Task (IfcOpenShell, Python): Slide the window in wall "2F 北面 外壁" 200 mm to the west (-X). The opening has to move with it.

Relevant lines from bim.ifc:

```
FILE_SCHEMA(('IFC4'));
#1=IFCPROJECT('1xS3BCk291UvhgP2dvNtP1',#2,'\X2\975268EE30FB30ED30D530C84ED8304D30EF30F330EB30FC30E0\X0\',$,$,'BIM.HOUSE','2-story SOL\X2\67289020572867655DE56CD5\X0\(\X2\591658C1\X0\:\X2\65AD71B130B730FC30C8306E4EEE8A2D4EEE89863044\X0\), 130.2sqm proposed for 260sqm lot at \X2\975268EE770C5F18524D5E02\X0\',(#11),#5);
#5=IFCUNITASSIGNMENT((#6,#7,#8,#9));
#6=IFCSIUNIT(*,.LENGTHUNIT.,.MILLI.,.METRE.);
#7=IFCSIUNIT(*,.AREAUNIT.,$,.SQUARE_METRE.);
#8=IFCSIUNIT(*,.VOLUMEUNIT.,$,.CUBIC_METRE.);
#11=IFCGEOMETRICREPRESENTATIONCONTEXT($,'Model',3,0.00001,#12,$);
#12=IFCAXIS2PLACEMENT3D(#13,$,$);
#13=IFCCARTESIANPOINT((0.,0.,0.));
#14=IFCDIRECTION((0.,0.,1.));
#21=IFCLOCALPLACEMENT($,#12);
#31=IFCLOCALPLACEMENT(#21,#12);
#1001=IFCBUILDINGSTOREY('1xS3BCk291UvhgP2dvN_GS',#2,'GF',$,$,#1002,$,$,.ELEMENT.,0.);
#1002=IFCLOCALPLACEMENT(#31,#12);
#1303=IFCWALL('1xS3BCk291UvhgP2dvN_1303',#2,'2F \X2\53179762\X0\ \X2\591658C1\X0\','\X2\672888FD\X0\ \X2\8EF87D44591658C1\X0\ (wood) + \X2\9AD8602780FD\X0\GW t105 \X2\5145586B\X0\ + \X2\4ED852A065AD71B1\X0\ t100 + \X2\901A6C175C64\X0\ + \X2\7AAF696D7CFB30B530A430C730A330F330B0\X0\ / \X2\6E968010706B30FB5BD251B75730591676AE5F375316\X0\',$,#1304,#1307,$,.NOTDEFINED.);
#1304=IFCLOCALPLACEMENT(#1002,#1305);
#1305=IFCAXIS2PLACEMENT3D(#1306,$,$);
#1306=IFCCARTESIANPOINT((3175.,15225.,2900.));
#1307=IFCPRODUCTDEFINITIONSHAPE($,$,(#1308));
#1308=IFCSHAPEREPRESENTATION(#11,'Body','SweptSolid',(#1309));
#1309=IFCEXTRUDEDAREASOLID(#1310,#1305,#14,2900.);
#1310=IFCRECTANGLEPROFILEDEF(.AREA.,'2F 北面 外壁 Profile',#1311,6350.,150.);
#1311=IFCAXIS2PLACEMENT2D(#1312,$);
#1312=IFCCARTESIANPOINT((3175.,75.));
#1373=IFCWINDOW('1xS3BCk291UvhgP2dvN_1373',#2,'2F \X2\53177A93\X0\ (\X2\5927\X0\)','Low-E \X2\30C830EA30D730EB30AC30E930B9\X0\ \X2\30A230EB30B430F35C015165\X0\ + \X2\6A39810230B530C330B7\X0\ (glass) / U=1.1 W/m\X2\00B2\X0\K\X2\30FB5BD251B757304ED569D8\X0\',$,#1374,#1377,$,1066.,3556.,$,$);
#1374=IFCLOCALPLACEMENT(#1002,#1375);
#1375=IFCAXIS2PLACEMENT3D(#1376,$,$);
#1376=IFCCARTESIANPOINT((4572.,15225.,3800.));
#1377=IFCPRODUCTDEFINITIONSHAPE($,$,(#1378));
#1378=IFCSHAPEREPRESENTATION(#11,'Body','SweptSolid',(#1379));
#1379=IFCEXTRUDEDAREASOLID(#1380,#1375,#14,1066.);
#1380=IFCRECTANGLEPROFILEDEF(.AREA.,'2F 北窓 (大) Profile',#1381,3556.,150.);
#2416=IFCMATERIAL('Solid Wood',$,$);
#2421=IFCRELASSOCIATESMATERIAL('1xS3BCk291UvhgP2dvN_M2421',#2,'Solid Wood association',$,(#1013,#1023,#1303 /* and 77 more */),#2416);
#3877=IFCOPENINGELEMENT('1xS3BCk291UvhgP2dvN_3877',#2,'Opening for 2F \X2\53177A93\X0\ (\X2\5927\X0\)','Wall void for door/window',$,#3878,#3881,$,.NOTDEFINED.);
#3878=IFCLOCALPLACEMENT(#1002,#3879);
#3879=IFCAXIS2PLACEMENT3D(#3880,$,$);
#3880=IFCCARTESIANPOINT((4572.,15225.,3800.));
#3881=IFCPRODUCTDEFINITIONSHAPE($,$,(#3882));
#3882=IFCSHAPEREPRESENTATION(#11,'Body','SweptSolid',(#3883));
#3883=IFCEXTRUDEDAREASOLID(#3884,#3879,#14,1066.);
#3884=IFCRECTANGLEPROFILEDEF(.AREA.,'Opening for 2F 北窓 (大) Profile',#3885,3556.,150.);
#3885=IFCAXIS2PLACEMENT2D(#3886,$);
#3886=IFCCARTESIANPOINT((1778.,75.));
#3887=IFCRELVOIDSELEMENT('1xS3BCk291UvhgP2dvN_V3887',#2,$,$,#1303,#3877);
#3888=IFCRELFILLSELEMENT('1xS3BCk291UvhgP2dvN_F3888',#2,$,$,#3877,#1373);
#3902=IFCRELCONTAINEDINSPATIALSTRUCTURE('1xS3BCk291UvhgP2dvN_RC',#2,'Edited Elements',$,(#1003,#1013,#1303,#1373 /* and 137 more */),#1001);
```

```python
import ifcopenshell
import ifcopenshell.api.geometry
import ifcopenshell.util.placement
import ifcopenshell.util.unit

model = ifcopenshell.open("bim.ifc")
unit_scale = ifcopenshell.util.unit.calculate_unit_scale(model)

window = model.by_guid("1xS3BCk291UvhgP2dvN_1373")
opening = window.FillsVoids[0].RelatingOpeningElement
wall = opening.VoidsElements[0].RelatingBuildingElement

wall_matrix = ifcopenshell.util.placement.get_local_placement(wall.ObjectPlacement)
shift = wall_matrix[:3, 0] * -0.2 / unit_scale
before = ifcopenshell.util.placement.get_local_placement(window.ObjectPlacement)[:3, 3].copy()

# The window is not placed relative to its opening, so move both.
for product in (opening, window):
    matrix = ifcopenshell.util.placement.get_local_placement(product.ObjectPlacement)
    matrix[:3, 3] += shift
    ifcopenshell.api.geometry.edit_object_placement(model, product=product, matrix=matrix, is_si=False)

after = ifcopenshell.util.placement.get_local_placement(window.ObjectPlacement)[:3, 3]
print("window moved by", (after - before).round(3) + 0.0)

model.write("bim_edited.ifc")
```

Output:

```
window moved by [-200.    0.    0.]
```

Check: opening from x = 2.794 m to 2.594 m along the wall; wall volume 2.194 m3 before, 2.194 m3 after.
